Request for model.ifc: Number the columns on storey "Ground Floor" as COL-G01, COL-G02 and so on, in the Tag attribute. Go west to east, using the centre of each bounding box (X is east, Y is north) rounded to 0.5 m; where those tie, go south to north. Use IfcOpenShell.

First a look at what the model holds.

```python
import ifcopenshell
import ifcopenshell.util.element
import ifcopenshell.util.placement

model = ifcopenshell.open("model.ifc")
print(model.schema)
storey = next(s for s in model.by_type("IfcBuildingStorey") if s.Name == "Ground Floor")
columns = [e for e in ifcopenshell.util.element.get_decomposition(storey) if e.is_a("IfcColumn")]
for e in sorted(columns, key=lambda e: e.id()):
    origin = ifcopenshell.util.placement.get_local_placement(e.ObjectPlacement)[:3, 3]
    print(e.id(), e.Tag, e.Name, origin.round(2) + 0.0, sep=" | ")
```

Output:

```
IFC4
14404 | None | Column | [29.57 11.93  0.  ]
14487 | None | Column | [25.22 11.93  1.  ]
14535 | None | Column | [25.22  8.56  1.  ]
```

```python
import ifcopenshell
import ifcopenshell.geom
import ifcopenshell.util.element
import ifcopenshell.util.shape

model = ifcopenshell.open("model.ifc")
settings = ifcopenshell.geom.settings()
settings.set("use-world-coords", True)


def centre(element):
    shape = ifcopenshell.geom.create_shape(settings, element)
    return ifcopenshell.util.shape.get_bbox_centroid(shape.geometry)


storey = next(s for s in model.by_type("IfcBuildingStorey") if s.Name == "Ground Floor")
columns = [e for e in ifcopenshell.util.element.get_decomposition(storey) if e.is_a("IfcColumn")]

# Insertion points can sit at a corner or the storey origin, so sort by the geometry (in metres).
centres = {e: centre(e) for e in columns}
columns.sort(key=lambda e: (round(centres[e][0] / 0.5), centres[e][1]))

for i, e in enumerate(columns, start=1):
    number = f"COL-G{i:02d}"
    e.Tag = number
    print(e.id(), number)

model.write("model_rev.ifc")
```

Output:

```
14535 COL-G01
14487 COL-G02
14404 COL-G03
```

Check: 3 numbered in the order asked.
